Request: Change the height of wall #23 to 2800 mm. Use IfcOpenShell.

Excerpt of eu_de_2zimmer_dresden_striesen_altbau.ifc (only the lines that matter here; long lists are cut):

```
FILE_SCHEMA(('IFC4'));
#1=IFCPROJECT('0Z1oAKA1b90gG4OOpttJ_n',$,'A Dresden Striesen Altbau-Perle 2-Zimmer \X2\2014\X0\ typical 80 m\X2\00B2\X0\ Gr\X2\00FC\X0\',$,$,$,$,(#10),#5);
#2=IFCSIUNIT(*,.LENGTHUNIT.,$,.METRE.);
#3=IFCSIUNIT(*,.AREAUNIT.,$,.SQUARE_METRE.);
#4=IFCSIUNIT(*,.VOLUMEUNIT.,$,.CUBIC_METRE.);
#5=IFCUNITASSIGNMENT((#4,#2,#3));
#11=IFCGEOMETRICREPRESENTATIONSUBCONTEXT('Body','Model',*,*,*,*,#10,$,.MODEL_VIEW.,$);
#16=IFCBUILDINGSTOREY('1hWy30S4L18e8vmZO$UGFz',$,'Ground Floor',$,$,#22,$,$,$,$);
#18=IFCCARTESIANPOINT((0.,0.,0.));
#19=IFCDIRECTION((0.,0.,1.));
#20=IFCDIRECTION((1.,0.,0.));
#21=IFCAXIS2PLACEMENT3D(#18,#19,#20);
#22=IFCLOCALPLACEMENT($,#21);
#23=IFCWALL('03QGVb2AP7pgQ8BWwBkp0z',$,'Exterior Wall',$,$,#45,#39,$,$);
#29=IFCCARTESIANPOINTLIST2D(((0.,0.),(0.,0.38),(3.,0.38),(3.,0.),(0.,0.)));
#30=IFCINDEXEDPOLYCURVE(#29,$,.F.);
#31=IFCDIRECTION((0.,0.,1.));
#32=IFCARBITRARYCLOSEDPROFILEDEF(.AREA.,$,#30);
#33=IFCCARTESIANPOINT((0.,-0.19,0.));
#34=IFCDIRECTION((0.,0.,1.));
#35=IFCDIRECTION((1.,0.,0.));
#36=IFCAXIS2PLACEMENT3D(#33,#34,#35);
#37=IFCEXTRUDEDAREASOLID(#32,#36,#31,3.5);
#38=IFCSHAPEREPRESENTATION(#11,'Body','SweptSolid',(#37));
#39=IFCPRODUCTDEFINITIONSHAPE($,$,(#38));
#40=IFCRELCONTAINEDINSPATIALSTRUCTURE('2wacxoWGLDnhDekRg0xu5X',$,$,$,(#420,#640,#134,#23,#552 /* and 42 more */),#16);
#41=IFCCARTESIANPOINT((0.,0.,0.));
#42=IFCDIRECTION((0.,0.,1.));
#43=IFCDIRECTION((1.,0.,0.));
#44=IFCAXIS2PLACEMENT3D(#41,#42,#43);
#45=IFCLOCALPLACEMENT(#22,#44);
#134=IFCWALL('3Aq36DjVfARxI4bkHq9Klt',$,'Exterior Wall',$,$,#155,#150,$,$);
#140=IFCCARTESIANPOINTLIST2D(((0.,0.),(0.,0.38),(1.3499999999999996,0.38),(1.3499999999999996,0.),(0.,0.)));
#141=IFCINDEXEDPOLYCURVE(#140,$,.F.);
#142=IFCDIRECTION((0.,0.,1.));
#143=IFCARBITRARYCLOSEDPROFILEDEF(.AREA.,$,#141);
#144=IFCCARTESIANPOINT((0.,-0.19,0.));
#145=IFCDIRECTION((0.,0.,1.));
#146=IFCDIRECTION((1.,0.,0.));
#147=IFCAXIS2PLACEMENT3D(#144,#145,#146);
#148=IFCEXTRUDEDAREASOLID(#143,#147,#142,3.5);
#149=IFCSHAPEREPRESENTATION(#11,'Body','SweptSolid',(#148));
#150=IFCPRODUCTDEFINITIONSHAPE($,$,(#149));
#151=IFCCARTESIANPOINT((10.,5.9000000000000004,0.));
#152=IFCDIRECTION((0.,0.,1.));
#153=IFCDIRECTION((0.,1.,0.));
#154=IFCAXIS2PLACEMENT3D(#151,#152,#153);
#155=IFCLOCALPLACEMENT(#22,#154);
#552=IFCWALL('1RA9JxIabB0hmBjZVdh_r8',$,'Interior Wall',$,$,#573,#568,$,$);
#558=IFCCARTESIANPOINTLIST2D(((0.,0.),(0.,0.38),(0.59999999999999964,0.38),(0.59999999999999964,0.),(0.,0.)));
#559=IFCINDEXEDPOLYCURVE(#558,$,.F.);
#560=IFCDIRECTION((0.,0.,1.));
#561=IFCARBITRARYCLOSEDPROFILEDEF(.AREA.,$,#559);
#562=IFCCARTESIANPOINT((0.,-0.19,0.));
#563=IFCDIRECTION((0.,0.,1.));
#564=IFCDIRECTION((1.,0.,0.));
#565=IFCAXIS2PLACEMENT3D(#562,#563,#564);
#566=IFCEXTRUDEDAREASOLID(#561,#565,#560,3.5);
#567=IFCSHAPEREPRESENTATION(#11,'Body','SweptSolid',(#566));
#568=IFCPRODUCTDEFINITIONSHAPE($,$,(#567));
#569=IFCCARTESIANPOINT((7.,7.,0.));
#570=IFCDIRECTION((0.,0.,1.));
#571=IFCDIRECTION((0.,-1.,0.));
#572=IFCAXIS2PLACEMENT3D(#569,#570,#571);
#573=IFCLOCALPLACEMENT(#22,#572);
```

```python
import ifcopenshell
import ifcopenshell.geom
import ifcopenshell.util.representation
import ifcopenshell.util.shape
import ifcopenshell.util.unit

model = ifcopenshell.open("eu_de_2zimmer_dresden_striesen_altbau.ifc")
unit_scale = ifcopenshell.util.unit.calculate_unit_scale(model)
settings = ifcopenshell.geom.settings()


def volume(element):
    """Net volume in cubic metres, openings subtracted."""
    shape = ifcopenshell.geom.create_shape(settings, element)
    return ifcopenshell.util.shape.get_volume(shape.geometry)


wall = model.by_guid("03QGVb2AP7pgQ8BWwBkp0z")
before = volume(wall)

body = ifcopenshell.util.representation.get_representation(wall, "Model", "Body")
solid = body.Items[0]
old_height = solid.Depth
solid.Depth = 2.8 / unit_scale
after = volume(wall)

print(f"height {old_height:g} -> {solid.Depth:g}, volume {before:.3f} -> {after:.3f} m3")

model.write("eu_de_2zimmer_dresden_striesen_altbau_edited.ifc")
```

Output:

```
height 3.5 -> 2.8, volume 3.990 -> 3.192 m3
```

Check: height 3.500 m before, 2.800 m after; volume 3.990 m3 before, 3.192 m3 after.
